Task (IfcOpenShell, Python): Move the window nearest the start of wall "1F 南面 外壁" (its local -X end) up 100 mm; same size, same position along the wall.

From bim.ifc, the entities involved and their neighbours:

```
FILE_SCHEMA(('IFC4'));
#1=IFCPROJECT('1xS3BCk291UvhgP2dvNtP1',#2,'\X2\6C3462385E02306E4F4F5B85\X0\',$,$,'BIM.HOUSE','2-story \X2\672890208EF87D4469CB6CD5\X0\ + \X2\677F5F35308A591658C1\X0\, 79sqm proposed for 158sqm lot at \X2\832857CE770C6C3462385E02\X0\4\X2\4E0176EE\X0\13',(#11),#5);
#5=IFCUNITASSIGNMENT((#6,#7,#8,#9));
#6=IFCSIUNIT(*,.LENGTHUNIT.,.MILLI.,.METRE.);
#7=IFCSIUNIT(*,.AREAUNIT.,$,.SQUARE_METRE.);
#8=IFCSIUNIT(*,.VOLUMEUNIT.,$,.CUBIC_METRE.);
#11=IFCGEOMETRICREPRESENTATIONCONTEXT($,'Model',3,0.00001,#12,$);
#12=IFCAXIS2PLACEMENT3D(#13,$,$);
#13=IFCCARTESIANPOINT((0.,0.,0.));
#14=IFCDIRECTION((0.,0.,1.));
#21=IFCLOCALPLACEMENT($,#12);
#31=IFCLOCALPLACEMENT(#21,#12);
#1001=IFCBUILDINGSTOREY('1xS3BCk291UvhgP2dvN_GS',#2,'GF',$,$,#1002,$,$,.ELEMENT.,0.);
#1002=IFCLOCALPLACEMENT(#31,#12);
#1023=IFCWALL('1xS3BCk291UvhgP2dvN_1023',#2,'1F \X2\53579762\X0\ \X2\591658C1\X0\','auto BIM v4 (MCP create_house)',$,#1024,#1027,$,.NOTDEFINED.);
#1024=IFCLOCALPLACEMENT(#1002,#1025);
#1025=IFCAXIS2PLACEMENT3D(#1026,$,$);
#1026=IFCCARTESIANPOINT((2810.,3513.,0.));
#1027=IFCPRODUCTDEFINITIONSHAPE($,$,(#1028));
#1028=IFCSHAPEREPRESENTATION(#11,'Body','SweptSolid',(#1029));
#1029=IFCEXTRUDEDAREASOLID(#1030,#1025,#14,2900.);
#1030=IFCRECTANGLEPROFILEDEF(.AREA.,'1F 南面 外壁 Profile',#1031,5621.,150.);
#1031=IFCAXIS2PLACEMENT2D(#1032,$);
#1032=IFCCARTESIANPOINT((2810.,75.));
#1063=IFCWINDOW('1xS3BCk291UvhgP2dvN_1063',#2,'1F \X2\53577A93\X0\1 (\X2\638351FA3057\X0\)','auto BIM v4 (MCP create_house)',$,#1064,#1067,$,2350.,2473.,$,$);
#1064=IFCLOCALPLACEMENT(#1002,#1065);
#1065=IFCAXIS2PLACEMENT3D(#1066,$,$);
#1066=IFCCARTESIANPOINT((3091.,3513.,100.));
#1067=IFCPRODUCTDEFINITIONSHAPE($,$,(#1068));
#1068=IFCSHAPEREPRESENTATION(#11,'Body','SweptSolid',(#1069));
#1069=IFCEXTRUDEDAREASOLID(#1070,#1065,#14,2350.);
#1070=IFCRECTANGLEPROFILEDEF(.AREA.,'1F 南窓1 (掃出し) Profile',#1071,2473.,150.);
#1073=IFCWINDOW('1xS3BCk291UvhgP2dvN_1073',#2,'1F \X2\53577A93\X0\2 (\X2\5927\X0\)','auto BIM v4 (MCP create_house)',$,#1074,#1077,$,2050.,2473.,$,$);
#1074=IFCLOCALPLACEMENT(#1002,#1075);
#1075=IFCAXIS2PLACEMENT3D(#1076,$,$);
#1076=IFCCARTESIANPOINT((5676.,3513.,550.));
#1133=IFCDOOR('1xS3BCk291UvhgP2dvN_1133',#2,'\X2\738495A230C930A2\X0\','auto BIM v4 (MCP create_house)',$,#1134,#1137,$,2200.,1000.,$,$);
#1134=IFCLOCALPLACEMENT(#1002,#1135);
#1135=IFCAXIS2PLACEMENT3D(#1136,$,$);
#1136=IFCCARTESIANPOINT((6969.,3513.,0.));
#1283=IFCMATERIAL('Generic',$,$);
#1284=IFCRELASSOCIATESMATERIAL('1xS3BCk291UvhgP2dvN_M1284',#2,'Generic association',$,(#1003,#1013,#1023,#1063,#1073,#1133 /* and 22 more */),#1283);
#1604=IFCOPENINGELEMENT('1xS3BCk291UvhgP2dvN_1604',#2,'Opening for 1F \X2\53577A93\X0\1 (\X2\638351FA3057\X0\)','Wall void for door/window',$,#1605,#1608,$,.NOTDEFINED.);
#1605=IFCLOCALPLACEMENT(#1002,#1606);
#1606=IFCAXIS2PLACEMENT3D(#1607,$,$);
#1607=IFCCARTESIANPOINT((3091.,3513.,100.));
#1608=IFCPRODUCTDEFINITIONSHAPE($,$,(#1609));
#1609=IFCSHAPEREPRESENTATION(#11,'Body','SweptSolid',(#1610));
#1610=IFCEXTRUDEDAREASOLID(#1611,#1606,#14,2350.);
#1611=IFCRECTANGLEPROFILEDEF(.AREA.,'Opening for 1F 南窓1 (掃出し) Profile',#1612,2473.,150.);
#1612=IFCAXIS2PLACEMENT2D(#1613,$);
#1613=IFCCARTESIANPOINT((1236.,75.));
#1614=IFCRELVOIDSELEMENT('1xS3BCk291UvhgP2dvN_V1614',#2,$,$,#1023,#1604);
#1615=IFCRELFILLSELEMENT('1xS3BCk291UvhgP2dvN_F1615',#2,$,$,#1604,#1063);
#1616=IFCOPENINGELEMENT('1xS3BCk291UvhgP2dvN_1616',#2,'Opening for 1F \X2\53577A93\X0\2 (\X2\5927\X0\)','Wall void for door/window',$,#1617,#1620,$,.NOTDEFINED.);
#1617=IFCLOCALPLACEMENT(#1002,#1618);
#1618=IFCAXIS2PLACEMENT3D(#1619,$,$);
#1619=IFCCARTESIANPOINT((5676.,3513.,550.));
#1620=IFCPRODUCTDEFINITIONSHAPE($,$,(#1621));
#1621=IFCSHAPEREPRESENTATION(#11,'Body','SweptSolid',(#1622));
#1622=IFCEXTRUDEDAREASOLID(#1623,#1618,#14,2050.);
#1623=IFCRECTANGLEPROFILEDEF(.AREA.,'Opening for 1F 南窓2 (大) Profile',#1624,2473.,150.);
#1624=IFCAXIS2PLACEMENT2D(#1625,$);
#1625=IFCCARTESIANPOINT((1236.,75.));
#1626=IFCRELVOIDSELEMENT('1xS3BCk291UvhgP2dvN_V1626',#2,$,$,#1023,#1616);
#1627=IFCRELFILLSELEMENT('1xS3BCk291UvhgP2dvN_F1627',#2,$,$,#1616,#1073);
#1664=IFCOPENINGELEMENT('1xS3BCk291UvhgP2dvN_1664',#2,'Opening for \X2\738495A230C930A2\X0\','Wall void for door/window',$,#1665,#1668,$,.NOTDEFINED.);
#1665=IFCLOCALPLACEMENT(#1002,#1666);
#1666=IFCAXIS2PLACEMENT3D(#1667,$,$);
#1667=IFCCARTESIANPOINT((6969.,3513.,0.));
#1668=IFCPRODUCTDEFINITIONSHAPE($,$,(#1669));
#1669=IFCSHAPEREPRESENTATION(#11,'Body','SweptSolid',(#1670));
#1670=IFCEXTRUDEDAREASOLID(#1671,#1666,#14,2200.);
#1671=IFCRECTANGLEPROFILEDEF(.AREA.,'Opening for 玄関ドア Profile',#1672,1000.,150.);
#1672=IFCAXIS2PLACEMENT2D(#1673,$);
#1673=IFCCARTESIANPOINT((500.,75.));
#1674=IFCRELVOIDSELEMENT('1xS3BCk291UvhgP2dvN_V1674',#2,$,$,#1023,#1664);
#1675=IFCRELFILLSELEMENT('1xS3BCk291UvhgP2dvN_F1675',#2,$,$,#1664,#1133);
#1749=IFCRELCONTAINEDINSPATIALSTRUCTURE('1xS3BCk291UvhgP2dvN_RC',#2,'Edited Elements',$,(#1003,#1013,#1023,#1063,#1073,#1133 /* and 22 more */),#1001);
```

```python
import numpy as np
import ifcopenshell
import ifcopenshell.api.geometry
import ifcopenshell.util.placement
import ifcopenshell.util.unit

model = ifcopenshell.open("bim.ifc")
unit_scale = ifcopenshell.util.unit.calculate_unit_scale(model)

window = model.by_id(1063)
opening = window.FillsVoids[0].RelatingOpeningElement
dz = 0.1 / unit_scale

shift = np.array([0.0, 0.0, dz])
# The window is not placed relative to its opening, so move both.
for product in (opening, window):
    matrix = ifcopenshell.util.placement.get_local_placement(product.ObjectPlacement)
    matrix[:3, 3] += shift
    ifcopenshell.api.geometry.edit_object_placement(model, product=product, matrix=matrix, is_si=False)

print(f"moved by {dz * unit_scale:+.3f} m")

model.write("bim_rev.ifc")
```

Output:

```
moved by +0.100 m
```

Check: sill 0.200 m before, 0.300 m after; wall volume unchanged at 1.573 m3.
